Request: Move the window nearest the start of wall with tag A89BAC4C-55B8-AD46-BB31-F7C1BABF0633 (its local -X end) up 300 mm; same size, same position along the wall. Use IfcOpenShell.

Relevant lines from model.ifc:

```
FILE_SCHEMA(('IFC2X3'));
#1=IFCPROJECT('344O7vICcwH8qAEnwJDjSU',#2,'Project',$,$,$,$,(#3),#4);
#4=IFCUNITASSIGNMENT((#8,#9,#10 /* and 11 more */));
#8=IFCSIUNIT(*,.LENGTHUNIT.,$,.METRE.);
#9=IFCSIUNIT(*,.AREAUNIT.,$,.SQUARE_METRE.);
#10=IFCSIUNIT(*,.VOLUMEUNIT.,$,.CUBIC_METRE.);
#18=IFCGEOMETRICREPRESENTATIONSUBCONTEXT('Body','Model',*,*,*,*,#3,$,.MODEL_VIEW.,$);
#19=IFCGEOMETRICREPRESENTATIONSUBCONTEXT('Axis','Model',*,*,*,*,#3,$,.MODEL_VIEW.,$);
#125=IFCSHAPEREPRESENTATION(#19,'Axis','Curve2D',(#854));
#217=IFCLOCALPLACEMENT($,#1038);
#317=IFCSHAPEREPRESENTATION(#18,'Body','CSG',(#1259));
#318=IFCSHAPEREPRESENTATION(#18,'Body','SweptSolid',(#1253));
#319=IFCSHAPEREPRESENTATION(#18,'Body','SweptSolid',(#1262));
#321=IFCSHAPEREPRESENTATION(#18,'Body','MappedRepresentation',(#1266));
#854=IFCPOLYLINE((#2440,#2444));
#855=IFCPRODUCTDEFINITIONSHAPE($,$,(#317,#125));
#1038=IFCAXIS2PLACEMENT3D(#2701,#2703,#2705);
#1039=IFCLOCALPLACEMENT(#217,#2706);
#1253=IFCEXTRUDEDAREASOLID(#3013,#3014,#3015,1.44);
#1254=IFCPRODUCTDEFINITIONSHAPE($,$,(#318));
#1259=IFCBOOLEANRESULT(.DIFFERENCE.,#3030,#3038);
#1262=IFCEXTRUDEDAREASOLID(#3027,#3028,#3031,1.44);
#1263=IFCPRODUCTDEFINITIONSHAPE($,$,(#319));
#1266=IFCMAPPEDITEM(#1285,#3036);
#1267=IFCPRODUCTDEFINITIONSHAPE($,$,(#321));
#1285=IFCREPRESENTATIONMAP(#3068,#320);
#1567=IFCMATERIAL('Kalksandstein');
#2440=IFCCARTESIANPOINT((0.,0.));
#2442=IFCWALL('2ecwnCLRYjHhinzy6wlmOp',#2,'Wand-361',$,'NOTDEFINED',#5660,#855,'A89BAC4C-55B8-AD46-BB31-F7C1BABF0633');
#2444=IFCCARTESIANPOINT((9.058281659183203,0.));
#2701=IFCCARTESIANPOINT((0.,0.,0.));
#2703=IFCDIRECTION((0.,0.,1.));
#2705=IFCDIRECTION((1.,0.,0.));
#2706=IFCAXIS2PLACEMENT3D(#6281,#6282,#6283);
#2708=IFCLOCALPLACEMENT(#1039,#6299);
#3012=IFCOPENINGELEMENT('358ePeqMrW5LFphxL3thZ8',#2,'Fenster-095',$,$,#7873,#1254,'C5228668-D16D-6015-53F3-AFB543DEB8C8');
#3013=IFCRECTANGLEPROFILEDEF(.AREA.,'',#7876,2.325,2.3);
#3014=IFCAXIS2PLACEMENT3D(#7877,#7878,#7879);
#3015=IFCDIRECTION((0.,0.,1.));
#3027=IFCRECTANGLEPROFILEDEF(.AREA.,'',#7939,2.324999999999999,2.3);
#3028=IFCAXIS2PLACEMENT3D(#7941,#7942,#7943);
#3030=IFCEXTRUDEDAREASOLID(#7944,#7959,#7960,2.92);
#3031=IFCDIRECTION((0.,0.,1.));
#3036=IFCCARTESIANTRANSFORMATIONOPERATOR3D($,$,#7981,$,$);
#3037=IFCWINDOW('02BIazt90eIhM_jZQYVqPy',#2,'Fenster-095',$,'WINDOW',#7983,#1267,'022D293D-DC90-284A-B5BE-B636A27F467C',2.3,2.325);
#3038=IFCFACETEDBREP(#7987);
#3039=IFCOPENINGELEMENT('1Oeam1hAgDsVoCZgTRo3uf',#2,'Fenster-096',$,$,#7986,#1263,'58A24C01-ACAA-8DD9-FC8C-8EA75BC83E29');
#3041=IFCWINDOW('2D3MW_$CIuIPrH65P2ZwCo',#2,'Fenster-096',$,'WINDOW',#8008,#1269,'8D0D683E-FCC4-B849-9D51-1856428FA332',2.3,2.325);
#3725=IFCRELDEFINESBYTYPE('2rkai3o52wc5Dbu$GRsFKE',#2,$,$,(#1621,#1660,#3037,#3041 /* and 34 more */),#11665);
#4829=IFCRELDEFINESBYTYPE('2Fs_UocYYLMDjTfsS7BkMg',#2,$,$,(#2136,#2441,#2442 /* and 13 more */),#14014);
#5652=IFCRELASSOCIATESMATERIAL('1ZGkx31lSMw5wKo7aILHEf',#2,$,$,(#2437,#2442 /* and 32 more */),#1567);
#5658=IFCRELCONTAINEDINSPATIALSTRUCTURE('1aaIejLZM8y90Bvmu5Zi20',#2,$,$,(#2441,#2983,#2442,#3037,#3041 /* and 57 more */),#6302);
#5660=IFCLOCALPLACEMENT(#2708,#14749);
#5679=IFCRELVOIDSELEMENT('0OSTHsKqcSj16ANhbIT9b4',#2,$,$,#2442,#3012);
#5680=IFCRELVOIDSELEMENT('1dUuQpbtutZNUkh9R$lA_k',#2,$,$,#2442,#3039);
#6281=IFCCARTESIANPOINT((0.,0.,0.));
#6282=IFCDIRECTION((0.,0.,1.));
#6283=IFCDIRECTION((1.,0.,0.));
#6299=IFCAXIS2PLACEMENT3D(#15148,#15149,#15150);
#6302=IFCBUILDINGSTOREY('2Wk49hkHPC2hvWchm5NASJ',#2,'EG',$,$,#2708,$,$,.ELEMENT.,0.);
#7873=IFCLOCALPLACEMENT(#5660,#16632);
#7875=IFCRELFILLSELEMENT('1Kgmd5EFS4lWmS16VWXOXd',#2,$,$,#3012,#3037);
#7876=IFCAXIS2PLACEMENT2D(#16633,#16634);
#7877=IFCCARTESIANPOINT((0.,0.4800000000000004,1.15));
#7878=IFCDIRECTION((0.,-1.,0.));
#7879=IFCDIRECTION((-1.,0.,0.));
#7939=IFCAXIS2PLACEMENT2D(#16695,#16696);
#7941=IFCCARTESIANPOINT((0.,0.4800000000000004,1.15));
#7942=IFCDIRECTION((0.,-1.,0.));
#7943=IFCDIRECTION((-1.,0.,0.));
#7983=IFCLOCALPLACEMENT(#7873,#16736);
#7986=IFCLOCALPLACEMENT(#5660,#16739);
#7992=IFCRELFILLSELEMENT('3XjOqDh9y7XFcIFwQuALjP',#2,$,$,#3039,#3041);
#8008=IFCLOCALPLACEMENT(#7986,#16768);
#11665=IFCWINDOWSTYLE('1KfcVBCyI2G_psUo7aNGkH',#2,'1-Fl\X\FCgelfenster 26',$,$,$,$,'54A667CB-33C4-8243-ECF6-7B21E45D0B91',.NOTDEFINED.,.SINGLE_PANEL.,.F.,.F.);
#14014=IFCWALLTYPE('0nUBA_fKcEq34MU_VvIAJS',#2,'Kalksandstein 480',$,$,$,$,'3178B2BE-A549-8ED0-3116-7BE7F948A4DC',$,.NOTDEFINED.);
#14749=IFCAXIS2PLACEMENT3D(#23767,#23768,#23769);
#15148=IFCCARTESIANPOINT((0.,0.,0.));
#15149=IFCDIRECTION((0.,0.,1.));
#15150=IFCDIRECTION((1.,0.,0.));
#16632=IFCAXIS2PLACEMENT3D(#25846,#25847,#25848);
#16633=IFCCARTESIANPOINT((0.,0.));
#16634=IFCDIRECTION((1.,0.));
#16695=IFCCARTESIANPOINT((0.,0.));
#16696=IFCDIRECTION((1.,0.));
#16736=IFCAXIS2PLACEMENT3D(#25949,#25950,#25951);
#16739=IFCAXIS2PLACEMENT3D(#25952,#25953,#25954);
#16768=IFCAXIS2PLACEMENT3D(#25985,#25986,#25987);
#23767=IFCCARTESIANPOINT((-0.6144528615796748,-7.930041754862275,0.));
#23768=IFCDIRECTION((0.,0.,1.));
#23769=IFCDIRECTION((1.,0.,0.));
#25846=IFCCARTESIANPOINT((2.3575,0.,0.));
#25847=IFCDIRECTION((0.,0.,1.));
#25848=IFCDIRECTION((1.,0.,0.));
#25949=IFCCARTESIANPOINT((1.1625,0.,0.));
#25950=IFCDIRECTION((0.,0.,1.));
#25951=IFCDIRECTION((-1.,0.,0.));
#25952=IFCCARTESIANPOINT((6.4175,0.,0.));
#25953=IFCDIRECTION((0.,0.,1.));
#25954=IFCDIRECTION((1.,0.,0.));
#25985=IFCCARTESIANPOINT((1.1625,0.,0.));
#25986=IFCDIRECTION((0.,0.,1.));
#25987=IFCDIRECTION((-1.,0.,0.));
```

```python
import numpy as np
import ifcopenshell
import ifcopenshell.api.geometry
import ifcopenshell.util.placement
import ifcopenshell.util.unit

model = ifcopenshell.open("model.ifc")
unit_scale = ifcopenshell.util.unit.calculate_unit_scale(model)

window = model.by_guid("02BIazt90eIhM_jZQYVqPy")
opening = window.FillsVoids[0].RelatingOpeningElement
dz = 0.3 / unit_scale

shift = np.array([0.0, 0.0, dz])
# The window is placed relative to its opening, so it follows when the opening moves.
matrix = ifcopenshell.util.placement.get_local_placement(opening.ObjectPlacement)
matrix[:3, 3] += shift
ifcopenshell.api.geometry.edit_object_placement(
    model, product=opening, matrix=matrix, is_si=False, should_transform_children=True
)

print(f"moved by {dz * unit_scale:+.3f} m")

model.write("model-out.ifc")
```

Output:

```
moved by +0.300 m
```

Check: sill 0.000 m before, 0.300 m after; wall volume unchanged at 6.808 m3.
